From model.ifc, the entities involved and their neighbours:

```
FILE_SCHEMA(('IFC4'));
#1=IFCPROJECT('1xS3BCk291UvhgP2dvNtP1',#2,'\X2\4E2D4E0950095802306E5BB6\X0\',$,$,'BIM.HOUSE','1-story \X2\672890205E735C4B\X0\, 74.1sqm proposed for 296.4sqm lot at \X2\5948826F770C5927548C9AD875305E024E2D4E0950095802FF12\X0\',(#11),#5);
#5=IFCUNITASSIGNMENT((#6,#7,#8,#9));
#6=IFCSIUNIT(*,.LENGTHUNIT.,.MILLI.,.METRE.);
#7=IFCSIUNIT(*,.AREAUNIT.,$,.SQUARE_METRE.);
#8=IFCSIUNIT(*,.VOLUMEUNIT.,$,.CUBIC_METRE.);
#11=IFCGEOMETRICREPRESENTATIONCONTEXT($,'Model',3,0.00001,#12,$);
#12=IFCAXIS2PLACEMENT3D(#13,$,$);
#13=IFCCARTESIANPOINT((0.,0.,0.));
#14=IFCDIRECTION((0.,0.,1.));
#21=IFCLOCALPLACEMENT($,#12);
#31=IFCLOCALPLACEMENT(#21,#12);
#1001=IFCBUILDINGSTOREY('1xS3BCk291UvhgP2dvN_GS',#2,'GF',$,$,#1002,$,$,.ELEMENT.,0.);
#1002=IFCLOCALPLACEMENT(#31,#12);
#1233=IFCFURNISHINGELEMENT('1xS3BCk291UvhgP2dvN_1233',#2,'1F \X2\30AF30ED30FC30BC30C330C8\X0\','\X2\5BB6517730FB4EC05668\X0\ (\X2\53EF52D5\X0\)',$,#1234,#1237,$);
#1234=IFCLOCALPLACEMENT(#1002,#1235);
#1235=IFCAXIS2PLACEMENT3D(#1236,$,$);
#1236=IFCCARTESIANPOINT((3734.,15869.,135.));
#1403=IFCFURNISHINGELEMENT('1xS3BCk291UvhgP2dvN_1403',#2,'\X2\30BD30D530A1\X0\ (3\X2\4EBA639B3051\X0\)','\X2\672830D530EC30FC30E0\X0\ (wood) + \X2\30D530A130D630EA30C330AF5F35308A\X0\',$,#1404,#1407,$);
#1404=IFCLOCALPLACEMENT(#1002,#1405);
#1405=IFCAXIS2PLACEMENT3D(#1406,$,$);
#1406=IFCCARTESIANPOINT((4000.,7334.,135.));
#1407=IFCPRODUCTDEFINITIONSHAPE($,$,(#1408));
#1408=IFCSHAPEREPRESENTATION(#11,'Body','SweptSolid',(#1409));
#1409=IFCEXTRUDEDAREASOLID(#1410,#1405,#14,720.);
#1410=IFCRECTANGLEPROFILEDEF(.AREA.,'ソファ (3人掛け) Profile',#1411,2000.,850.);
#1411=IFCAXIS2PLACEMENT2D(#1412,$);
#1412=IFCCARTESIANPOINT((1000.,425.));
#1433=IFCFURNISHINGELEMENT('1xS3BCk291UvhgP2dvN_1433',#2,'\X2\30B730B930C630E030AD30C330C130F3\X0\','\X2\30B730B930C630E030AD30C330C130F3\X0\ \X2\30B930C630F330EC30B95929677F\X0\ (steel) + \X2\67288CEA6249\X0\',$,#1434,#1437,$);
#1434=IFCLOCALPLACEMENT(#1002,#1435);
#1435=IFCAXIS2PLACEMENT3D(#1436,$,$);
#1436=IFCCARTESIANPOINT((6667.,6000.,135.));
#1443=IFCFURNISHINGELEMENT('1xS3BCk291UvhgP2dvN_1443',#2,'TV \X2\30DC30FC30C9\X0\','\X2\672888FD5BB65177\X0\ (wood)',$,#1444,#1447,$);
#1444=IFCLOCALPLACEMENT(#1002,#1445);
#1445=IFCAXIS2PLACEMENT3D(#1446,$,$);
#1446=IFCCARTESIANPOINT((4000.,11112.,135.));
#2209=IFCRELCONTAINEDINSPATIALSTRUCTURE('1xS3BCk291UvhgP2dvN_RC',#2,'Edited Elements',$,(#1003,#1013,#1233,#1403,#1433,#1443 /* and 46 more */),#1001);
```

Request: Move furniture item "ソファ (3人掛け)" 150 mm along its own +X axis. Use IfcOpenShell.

```python
import ifcopenshell
import ifcopenshell.api.geometry
import ifcopenshell.util.placement
import ifcopenshell.util.unit

model = ifcopenshell.open("model.ifc")
unit_scale = ifcopenshell.util.unit.calculate_unit_scale(model)

item = model.by_guid("1xS3BCk291UvhgP2dvN_1403")
matrix = ifcopenshell.util.placement.get_local_placement(item.ObjectPlacement)
matrix[:3, 3] += matrix[:3, 0] * 0.15 / unit_scale
ifcopenshell.api.geometry.edit_object_placement(model, product=item, matrix=matrix, is_si=False)

print(ifcopenshell.util.placement.get_local_placement(item.ObjectPlacement).round(3) + 0.0)

model.write("model_updated.ifc")
```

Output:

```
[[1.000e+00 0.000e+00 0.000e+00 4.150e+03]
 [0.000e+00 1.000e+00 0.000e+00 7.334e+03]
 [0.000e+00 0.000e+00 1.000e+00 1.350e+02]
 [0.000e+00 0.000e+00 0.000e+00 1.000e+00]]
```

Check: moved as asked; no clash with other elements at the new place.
